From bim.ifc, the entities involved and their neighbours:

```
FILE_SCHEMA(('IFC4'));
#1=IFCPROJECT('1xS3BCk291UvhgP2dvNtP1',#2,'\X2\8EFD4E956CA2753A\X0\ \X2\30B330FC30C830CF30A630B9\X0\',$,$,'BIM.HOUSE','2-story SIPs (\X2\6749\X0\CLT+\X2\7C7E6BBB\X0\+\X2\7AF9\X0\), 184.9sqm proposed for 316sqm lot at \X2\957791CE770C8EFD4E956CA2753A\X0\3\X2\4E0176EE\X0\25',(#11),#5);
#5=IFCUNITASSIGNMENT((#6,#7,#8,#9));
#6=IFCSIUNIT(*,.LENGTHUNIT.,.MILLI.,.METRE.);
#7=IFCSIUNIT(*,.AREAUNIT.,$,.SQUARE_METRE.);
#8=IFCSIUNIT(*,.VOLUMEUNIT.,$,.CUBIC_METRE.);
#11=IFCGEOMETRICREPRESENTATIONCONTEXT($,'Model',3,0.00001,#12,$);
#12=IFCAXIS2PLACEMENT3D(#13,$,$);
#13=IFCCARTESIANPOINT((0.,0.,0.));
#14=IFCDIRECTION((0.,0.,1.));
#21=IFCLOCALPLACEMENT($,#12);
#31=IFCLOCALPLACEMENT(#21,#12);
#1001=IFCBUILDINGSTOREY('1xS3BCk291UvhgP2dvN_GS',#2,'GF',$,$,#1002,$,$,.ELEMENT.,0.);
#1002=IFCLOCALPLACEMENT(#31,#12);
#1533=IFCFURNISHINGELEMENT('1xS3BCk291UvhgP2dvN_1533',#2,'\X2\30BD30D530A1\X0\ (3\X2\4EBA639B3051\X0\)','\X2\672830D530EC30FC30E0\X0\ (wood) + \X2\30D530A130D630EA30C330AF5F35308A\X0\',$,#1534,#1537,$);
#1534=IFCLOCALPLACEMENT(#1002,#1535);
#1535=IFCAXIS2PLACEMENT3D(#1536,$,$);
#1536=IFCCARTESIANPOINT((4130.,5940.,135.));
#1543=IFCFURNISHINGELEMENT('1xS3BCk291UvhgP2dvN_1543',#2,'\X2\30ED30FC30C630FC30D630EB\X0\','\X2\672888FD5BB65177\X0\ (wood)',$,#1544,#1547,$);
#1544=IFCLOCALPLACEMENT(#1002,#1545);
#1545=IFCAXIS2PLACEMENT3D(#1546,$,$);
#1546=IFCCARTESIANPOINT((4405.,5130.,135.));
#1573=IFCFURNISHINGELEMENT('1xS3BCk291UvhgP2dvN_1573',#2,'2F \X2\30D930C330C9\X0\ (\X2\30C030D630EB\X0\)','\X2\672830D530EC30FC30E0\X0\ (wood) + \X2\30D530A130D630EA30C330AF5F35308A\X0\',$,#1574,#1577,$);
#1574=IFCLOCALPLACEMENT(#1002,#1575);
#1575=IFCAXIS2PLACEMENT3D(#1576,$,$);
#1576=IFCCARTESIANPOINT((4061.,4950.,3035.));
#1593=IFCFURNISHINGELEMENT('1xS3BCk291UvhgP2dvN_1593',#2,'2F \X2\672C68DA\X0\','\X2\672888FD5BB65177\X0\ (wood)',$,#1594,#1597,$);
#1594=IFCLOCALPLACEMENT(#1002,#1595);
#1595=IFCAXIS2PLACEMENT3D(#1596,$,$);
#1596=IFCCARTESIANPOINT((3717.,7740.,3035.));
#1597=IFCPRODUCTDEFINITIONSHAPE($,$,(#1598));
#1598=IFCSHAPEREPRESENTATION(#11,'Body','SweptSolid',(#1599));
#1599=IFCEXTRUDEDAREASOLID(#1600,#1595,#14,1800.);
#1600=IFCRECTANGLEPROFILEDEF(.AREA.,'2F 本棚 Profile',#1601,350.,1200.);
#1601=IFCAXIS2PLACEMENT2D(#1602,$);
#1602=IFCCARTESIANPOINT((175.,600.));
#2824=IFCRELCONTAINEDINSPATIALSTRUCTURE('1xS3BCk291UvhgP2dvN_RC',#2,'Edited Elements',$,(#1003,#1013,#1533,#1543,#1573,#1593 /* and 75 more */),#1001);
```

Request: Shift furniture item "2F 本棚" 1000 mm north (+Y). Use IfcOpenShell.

```python
import ifcopenshell
import ifcopenshell.api.geometry
import ifcopenshell.util.placement

model = ifcopenshell.open("bim.ifc")

item = model.by_guid("1xS3BCk291UvhgP2dvN_1593")
matrix = ifcopenshell.util.placement.get_local_placement(item.ObjectPlacement)
matrix[1, 3] += 1000.0
ifcopenshell.api.geometry.edit_object_placement(model, product=item, matrix=matrix, is_si=False)

print(ifcopenshell.util.placement.get_local_placement(item.ObjectPlacement).round(3) + 0.0)

model.write("bim-out.ifc")
```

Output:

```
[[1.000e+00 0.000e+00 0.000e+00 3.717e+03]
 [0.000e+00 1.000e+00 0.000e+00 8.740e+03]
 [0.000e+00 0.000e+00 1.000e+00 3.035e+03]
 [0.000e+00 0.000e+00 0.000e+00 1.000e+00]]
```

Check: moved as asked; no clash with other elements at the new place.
